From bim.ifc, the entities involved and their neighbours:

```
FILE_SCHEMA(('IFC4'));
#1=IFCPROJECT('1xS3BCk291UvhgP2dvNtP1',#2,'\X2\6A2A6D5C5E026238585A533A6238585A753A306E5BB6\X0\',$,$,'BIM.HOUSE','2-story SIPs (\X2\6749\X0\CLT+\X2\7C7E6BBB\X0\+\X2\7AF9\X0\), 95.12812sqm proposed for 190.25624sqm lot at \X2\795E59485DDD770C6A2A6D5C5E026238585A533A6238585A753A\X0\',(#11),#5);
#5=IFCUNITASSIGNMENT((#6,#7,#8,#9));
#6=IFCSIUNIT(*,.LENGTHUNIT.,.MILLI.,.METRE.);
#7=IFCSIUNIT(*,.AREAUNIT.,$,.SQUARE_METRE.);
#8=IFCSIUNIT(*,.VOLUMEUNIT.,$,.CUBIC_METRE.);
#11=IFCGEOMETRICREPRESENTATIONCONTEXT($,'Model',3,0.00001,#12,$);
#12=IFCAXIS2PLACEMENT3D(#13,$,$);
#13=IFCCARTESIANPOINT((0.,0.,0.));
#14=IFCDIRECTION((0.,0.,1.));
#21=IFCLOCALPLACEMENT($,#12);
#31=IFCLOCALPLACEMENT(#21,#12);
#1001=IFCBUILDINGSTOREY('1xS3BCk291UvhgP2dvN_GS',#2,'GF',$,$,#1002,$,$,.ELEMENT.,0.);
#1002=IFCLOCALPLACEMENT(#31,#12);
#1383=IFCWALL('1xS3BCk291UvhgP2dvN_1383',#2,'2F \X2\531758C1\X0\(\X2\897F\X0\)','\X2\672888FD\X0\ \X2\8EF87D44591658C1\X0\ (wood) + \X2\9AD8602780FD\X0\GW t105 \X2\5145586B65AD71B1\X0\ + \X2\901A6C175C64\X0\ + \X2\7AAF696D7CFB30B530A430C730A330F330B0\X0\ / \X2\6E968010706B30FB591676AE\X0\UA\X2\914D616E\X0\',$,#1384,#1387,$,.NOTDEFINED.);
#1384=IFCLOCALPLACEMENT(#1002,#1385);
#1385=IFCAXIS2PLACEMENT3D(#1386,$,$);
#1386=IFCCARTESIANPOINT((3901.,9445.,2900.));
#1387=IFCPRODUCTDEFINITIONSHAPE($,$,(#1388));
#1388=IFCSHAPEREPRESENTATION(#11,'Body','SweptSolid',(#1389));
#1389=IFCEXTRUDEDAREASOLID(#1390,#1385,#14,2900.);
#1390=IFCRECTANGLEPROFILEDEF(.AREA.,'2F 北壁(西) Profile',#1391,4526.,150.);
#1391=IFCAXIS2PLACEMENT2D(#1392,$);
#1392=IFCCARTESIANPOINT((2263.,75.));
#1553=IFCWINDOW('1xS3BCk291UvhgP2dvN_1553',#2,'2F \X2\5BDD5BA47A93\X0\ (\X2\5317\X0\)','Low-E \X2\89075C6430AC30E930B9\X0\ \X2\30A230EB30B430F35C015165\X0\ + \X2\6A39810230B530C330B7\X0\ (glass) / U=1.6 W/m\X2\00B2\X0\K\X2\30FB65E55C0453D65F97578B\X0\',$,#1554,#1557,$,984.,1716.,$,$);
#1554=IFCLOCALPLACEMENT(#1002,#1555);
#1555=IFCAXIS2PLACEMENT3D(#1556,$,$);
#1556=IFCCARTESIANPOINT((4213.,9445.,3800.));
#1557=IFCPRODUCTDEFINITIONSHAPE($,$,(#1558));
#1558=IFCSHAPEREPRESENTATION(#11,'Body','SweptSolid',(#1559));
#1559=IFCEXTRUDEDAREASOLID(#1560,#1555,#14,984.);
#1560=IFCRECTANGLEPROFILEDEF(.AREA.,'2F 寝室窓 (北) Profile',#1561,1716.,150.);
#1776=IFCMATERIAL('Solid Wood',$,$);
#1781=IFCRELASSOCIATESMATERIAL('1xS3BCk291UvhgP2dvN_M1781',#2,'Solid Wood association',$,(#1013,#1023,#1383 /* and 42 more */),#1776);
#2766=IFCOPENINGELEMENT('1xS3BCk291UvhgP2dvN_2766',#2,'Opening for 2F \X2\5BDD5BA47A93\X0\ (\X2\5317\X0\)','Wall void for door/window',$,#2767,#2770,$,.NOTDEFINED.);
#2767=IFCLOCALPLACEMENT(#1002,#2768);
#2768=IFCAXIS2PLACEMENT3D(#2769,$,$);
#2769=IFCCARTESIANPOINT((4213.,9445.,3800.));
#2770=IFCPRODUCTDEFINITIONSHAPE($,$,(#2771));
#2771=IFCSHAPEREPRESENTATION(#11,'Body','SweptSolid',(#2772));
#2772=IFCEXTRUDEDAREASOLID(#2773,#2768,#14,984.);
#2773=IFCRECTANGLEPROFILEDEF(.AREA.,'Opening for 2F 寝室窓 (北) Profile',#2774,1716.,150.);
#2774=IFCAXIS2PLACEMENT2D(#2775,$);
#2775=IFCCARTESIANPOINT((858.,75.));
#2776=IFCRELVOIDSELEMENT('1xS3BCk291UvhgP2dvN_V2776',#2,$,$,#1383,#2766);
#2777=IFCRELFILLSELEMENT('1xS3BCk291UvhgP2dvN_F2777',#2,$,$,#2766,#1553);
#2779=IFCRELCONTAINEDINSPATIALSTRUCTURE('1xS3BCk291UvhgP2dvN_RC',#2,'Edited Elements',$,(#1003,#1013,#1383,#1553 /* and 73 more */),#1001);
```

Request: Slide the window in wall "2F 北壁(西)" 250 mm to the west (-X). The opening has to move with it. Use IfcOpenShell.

```python
import ifcopenshell
import ifcopenshell.api.geometry
import ifcopenshell.util.placement
import ifcopenshell.util.unit

model = ifcopenshell.open("bim.ifc")
unit_scale = ifcopenshell.util.unit.calculate_unit_scale(model)

window = model.by_id(1553)
opening = window.FillsVoids[0].RelatingOpeningElement
wall = opening.VoidsElements[0].RelatingBuildingElement

wall_matrix = ifcopenshell.util.placement.get_local_placement(wall.ObjectPlacement)
shift = wall_matrix[:3, 0] * -0.25 / unit_scale
before = ifcopenshell.util.placement.get_local_placement(window.ObjectPlacement)[:3, 3].copy()

# The window is not placed relative to its opening, so move both.
for product in (opening, window):
    matrix = ifcopenshell.util.placement.get_local_placement(product.ObjectPlacement)
    matrix[:3, 3] += shift
    ifcopenshell.api.geometry.edit_object_placement(model, product=product, matrix=matrix, is_si=False)

after = ifcopenshell.util.placement.get_local_placement(window.ObjectPlacement)[:3, 3]
print("window moved by", (after - before).round(3) + 0.0)

model.write("bim_updated.ifc")
```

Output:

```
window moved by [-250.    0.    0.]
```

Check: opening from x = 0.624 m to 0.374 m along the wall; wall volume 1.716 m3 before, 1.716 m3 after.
